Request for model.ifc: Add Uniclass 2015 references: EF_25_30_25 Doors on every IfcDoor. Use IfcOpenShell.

First a look at what the model holds.

```python
import ifcopenshell

model = ifcopenshell.open("model.ifc")
print(model.schema)
print("classifications:", [c.Name for c in model.by_type("IfcClassification")])
for ifc_class in ("IfcDoor", "IfcRoof", "IfcStair", "IfcWall", "IfcWindow"):
    print(ifc_class, len(model.by_type(ifc_class)))
```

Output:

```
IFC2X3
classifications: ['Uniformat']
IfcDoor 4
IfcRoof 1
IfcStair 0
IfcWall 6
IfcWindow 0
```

```python
import ifcopenshell
import ifcopenshell.api.classification

model = ifcopenshell.open("model.ifc")

# IFC2X3 requires Source and Edition and has no link from the project to the system.
system = model.create_entity("IfcClassification", Source="NBS", Edition="2015", Name="Uniclass 2015")

codes = {
    "IfcDoor": ("EF_25_30_25", "Doors"),
}
for ifc_class, (code, name) in codes.items():
    products = model.by_type(ifc_class)
    ifcopenshell.api.classification.add_reference(
        model, products=products, classification=system, identification=code, name=name
    )
    print(code, len(products))

model.write("model_updated.ifc")
```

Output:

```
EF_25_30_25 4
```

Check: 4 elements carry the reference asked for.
